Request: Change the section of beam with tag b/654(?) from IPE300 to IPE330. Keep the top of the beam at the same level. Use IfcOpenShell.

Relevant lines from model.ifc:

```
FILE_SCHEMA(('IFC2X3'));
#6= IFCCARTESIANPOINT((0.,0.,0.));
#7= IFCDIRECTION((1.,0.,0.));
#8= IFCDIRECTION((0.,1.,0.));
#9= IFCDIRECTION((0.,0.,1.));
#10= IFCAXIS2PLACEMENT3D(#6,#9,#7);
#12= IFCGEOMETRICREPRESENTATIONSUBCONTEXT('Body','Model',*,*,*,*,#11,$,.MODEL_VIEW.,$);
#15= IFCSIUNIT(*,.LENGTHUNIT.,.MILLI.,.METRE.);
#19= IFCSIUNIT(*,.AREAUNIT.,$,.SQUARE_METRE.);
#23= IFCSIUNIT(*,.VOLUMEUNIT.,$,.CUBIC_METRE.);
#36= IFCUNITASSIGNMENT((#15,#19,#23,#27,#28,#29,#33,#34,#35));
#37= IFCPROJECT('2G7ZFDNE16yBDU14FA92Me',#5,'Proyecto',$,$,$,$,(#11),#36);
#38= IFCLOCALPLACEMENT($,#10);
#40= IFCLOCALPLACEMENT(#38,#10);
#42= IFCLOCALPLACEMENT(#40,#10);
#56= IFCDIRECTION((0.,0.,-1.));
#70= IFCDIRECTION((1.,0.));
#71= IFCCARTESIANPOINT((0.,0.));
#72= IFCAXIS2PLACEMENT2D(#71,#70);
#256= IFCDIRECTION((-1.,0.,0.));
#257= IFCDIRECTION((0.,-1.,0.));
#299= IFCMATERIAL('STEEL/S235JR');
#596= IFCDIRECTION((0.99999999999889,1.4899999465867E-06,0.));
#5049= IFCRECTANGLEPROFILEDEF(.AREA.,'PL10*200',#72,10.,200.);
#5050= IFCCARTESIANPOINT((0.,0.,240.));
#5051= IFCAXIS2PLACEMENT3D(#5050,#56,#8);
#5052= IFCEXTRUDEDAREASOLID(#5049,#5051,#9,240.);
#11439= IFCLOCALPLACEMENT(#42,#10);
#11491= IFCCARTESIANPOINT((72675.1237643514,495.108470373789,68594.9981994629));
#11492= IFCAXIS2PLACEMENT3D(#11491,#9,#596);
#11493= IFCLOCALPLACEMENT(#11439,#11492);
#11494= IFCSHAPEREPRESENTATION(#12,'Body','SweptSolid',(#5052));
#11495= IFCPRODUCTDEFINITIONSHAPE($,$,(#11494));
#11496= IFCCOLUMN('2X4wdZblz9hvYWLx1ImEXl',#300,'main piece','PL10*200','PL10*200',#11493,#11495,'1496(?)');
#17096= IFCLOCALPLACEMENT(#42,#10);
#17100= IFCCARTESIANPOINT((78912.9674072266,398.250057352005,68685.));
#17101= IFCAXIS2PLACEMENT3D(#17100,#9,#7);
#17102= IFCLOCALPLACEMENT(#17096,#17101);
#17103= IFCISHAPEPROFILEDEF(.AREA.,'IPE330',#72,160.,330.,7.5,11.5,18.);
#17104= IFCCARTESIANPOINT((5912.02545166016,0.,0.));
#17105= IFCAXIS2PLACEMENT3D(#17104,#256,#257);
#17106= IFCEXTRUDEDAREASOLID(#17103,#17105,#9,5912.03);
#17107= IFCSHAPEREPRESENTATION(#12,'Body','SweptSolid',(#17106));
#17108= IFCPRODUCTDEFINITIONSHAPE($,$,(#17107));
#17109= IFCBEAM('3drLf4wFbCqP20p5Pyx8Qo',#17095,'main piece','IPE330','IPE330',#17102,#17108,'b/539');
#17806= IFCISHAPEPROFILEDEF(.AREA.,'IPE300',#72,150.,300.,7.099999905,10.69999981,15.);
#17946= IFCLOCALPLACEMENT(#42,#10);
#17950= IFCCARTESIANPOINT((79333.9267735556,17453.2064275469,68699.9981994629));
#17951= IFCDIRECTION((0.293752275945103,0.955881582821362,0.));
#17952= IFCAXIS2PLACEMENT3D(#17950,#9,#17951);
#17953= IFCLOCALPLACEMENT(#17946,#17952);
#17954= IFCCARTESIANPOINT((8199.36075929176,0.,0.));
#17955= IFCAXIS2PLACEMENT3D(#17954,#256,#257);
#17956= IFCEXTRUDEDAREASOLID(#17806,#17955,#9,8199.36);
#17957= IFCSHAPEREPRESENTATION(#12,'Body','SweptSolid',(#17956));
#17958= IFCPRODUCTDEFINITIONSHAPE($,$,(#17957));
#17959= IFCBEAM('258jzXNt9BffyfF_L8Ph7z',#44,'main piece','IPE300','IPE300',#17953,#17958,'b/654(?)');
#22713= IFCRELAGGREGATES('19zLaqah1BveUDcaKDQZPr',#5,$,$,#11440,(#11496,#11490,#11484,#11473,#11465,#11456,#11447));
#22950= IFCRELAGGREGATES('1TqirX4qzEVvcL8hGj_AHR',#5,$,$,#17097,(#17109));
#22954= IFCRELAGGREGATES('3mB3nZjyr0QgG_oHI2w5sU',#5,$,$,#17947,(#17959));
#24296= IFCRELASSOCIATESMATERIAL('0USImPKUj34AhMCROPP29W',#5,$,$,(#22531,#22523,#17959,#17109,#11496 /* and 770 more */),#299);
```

```python
import ifcopenshell
import ifcopenshell.util.element
import ifcopenshell.util.representation

model = ifcopenshell.open("model.ifc")

member = model.by_id(17959)
source = next(p for p in model.by_type("IfcIShapeProfileDef") if p.ProfileName == "IPE330")

body = ifcopenshell.util.representation.get_representation(member, "Model", "Body")
solid = body.Items[0]
old_profile = solid.SweptArea

# Copy the section's sizes but keep this member's own profile position.
profile = ifcopenshell.util.element.copy(model, source)
# Profiles are centred, so shift by half the change in depth to hold the top.
shift = (old_profile.OverallDepth - profile.OverallDepth) / 2
x, y = old_profile.Position.Location.Coordinates
up = (0.0, 1.0)  # upwards, in the solid's own plane
location = model.createIfcCartesianPoint((x + up[0] * shift, y + up[1] * shift))
profile.Position = model.createIfcAxis2Placement2D(location, old_profile.Position.RefDirection)
solid.SweptArea = profile
if not model.get_total_inverses(old_profile):
    ifcopenshell.util.element.remove_deep2(model, old_profile)
member.Description = member.Description.replace("IPE300", "IPE330")
member.ObjectType = member.ObjectType.replace("IPE300", "IPE330")

print(solid.SweptArea)

model.write("model_updated.ifc")
```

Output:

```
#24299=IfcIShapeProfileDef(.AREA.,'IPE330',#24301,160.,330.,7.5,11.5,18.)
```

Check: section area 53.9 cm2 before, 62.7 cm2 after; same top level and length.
